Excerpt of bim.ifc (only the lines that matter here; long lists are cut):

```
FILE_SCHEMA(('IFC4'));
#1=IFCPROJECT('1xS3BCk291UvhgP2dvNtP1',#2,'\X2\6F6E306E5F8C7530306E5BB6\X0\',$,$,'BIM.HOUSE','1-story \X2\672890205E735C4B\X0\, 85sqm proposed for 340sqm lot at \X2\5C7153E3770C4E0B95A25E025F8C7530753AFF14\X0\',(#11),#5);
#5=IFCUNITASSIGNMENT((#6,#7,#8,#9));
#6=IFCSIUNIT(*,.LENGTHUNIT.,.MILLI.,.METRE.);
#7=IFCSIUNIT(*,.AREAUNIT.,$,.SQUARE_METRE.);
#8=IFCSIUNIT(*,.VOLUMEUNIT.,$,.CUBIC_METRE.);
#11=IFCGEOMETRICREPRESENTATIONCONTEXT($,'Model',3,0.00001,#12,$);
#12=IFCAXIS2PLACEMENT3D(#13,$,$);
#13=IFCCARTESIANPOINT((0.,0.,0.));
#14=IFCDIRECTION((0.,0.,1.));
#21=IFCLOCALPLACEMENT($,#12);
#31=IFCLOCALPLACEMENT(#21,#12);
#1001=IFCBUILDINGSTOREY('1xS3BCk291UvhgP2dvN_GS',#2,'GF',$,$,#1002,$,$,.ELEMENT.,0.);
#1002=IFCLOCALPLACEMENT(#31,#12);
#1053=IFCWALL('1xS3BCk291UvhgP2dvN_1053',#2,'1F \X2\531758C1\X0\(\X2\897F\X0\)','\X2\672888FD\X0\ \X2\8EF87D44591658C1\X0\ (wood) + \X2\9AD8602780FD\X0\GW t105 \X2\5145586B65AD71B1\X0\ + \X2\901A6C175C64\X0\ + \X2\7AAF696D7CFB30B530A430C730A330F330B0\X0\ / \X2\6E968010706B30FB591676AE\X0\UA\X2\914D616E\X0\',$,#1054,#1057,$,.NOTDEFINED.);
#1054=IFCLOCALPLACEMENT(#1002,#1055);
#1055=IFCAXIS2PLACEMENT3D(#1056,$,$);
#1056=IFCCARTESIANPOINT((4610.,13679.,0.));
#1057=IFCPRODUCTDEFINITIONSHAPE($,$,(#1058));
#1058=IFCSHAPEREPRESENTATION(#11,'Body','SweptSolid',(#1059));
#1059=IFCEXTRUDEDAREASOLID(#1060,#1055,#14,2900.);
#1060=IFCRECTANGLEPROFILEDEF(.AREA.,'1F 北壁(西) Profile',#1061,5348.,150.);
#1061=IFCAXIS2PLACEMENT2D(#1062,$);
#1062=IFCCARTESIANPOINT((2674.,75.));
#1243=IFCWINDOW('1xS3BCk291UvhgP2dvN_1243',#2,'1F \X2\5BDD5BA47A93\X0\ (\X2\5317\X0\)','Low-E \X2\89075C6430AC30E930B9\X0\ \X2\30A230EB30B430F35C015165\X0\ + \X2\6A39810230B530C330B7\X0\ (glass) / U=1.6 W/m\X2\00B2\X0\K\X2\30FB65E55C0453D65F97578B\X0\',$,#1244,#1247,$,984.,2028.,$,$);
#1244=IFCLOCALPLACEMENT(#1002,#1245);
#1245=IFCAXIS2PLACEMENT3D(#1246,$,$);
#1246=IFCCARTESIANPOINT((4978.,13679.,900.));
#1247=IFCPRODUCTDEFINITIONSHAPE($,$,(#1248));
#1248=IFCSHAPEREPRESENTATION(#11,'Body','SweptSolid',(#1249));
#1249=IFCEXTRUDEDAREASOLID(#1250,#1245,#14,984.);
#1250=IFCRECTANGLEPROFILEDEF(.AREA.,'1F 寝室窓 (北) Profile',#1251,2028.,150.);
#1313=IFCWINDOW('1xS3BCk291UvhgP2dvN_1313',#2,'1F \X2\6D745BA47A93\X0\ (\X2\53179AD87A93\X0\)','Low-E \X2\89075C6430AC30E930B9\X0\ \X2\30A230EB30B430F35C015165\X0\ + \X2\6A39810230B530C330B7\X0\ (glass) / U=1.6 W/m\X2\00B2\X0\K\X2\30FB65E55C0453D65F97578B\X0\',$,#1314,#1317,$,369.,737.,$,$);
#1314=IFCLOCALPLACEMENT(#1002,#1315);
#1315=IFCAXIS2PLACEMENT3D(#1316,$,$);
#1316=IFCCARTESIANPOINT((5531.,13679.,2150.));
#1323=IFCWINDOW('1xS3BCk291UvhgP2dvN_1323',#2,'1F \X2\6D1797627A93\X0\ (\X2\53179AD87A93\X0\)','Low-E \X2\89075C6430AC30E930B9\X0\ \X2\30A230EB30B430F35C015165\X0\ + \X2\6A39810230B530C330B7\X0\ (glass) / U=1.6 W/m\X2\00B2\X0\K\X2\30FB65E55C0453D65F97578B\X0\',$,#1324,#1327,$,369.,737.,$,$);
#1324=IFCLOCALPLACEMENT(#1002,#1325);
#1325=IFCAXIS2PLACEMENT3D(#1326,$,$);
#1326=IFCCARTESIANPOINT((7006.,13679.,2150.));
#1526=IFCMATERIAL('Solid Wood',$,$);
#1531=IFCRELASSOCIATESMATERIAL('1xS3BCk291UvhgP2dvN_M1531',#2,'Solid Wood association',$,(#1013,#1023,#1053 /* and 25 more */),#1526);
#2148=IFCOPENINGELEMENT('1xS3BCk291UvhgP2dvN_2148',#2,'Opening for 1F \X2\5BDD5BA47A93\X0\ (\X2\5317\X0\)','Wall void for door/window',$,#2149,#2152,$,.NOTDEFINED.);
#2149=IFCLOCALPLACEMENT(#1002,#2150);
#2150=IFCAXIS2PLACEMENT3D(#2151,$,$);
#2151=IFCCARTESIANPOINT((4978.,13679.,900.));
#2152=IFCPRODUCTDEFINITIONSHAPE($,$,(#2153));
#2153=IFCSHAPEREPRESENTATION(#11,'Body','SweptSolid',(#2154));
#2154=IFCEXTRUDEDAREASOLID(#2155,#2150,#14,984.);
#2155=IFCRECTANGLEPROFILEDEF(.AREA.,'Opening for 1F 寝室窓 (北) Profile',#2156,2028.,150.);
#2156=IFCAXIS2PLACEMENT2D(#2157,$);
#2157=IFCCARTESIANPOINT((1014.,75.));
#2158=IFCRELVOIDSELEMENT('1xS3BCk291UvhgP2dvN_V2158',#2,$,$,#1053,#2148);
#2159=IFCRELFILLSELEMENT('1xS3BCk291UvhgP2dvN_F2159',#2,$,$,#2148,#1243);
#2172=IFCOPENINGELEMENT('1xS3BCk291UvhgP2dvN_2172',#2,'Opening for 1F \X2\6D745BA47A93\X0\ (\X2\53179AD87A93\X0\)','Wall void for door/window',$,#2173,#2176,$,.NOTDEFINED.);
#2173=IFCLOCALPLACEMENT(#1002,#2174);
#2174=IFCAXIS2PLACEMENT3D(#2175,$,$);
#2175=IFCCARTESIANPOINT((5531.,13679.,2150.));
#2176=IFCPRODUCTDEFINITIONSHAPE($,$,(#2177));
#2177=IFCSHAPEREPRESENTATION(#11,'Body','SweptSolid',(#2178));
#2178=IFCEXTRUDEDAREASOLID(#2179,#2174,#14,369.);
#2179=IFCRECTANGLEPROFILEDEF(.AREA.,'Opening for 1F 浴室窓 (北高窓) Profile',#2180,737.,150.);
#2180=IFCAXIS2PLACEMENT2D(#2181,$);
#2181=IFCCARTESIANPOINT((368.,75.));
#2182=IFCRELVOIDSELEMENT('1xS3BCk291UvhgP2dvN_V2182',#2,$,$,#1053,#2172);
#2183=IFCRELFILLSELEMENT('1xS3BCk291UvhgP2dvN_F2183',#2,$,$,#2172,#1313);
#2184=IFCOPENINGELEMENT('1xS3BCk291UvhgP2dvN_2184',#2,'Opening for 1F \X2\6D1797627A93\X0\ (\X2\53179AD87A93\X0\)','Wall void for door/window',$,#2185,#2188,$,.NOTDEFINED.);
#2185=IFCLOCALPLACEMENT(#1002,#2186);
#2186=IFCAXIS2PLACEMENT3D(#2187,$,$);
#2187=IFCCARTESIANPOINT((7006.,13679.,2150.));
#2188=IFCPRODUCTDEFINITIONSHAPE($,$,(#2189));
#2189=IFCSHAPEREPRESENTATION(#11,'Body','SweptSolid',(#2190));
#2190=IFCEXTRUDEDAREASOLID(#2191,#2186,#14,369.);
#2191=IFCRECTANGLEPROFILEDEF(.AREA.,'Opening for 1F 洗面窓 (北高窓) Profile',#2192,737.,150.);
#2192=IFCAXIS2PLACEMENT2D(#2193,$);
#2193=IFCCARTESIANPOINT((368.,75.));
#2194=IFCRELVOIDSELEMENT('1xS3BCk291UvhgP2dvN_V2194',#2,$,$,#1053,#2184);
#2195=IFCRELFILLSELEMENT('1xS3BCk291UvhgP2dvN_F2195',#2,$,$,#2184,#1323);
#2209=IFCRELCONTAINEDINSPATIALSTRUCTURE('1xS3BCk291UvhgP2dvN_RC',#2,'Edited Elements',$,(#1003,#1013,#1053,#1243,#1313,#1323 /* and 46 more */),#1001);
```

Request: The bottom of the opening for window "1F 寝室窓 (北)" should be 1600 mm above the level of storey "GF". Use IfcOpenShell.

```python
import numpy as np
import ifcopenshell
import ifcopenshell.api.geometry
import ifcopenshell.geom
import ifcopenshell.util.element
import ifcopenshell.util.placement
import ifcopenshell.util.shape
import ifcopenshell.util.unit

model = ifcopenshell.open("bim.ifc")
unit_scale = ifcopenshell.util.unit.calculate_unit_scale(model)

window = model.by_guid("1xS3BCk291UvhgP2dvN_1243")
opening = window.FillsVoids[0].RelatingOpeningElement
storey = ifcopenshell.util.element.get_container(window, ifc_class="IfcBuildingStorey")
level = ifcopenshell.util.placement.get_local_placement(storey.ObjectPlacement)[2, 3]

# The opening's origin need not be at the sill, so measure its lowest point.
shape = ifcopenshell.geom.create_shape(ifcopenshell.geom.settings(), opening)
bottom = ifcopenshell.util.shape.get_shape_bottom_elevation(shape, shape.geometry) / unit_scale
dz = level + 1.6 / unit_scale - bottom

shift = np.array([0.0, 0.0, dz])
# The window is not placed relative to its opening, so move both.
for product in (opening, window):
    matrix = ifcopenshell.util.placement.get_local_placement(product.ObjectPlacement)
    matrix[:3, 3] += shift
    ifcopenshell.api.geometry.edit_object_placement(model, product=product, matrix=matrix, is_si=False)

print(f"moved by {dz * unit_scale:+.3f} m")

model.write("bim_v2.ifc")
```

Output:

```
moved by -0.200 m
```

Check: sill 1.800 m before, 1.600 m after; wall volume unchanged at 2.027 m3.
